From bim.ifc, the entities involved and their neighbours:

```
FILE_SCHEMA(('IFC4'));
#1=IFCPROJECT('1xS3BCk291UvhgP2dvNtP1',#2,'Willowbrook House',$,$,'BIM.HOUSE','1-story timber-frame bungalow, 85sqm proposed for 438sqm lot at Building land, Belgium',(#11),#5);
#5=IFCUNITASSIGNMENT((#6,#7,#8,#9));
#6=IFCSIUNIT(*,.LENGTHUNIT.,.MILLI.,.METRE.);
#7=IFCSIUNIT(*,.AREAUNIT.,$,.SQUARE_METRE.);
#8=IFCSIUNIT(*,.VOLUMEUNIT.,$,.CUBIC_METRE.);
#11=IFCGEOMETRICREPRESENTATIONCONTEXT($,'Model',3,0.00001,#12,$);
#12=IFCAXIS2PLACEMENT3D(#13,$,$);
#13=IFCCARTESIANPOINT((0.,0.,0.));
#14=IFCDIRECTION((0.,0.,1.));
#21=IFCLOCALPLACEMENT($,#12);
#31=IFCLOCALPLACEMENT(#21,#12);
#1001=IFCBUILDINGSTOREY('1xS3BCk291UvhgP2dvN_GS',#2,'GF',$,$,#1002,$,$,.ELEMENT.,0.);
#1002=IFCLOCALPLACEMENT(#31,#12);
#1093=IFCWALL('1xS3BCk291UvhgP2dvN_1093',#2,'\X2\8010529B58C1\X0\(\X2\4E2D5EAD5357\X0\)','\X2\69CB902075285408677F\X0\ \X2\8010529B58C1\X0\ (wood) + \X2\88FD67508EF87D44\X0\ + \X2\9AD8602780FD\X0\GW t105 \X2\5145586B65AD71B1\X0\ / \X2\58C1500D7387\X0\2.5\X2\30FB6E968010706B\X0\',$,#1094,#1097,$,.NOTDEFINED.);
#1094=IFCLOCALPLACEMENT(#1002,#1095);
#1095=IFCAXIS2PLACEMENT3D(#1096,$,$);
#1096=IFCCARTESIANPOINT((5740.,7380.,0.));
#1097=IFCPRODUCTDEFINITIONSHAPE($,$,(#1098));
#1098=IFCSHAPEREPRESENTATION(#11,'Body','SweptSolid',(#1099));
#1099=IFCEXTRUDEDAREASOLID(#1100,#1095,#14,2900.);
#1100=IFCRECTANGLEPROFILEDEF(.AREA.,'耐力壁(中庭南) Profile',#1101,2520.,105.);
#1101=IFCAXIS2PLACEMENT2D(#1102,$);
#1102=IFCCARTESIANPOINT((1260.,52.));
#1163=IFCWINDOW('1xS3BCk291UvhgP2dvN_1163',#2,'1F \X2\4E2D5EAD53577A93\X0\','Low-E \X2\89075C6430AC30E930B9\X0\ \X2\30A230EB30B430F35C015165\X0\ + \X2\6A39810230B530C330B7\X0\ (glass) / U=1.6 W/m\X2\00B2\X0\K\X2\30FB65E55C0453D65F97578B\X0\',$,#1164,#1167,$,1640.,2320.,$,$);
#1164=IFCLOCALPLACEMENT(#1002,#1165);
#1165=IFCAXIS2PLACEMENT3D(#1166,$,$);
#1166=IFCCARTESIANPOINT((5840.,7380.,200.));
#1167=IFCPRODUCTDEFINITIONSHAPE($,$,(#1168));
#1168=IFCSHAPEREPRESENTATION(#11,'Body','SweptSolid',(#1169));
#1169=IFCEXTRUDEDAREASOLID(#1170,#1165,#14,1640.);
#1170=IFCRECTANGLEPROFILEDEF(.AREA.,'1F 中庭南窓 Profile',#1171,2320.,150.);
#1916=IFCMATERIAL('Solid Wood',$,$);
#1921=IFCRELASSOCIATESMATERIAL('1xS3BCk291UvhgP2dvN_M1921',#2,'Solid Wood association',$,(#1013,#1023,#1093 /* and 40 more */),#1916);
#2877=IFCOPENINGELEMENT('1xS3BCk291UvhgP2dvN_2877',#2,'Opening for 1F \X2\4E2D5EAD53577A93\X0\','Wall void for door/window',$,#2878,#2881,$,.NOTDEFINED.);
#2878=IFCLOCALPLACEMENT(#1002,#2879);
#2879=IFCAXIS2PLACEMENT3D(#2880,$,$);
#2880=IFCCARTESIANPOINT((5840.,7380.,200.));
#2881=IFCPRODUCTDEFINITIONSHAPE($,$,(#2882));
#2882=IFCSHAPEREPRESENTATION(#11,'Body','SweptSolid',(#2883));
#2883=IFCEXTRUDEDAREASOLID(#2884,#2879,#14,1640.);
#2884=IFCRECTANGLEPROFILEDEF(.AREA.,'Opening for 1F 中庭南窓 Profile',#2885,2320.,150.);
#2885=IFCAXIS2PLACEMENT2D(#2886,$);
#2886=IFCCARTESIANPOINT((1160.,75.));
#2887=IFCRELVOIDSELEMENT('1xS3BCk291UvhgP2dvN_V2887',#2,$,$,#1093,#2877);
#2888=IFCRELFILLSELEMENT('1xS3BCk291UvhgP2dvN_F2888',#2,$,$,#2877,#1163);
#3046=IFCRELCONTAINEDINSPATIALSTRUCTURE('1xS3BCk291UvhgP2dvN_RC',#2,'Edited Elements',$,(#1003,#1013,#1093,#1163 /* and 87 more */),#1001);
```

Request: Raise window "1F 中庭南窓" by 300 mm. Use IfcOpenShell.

```python
import numpy as np
import ifcopenshell
import ifcopenshell.api.geometry
import ifcopenshell.util.placement
import ifcopenshell.util.unit

model = ifcopenshell.open("bim.ifc")
unit_scale = ifcopenshell.util.unit.calculate_unit_scale(model)

window = model.by_guid("1xS3BCk291UvhgP2dvN_1163")
opening = window.FillsVoids[0].RelatingOpeningElement
dz = 300.0

shift = np.array([0.0, 0.0, dz])
# The window is not placed relative to its opening, so move both.
for product in (opening, window):
    matrix = ifcopenshell.util.placement.get_local_placement(product.ObjectPlacement)
    matrix[:3, 3] += shift
    ifcopenshell.api.geometry.edit_object_placement(model, product=product, matrix=matrix, is_si=False)

print(f"moved by {dz * unit_scale:+.3f} m")

model.write("bim_updated.ifc")
```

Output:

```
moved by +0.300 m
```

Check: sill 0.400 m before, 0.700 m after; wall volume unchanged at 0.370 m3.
